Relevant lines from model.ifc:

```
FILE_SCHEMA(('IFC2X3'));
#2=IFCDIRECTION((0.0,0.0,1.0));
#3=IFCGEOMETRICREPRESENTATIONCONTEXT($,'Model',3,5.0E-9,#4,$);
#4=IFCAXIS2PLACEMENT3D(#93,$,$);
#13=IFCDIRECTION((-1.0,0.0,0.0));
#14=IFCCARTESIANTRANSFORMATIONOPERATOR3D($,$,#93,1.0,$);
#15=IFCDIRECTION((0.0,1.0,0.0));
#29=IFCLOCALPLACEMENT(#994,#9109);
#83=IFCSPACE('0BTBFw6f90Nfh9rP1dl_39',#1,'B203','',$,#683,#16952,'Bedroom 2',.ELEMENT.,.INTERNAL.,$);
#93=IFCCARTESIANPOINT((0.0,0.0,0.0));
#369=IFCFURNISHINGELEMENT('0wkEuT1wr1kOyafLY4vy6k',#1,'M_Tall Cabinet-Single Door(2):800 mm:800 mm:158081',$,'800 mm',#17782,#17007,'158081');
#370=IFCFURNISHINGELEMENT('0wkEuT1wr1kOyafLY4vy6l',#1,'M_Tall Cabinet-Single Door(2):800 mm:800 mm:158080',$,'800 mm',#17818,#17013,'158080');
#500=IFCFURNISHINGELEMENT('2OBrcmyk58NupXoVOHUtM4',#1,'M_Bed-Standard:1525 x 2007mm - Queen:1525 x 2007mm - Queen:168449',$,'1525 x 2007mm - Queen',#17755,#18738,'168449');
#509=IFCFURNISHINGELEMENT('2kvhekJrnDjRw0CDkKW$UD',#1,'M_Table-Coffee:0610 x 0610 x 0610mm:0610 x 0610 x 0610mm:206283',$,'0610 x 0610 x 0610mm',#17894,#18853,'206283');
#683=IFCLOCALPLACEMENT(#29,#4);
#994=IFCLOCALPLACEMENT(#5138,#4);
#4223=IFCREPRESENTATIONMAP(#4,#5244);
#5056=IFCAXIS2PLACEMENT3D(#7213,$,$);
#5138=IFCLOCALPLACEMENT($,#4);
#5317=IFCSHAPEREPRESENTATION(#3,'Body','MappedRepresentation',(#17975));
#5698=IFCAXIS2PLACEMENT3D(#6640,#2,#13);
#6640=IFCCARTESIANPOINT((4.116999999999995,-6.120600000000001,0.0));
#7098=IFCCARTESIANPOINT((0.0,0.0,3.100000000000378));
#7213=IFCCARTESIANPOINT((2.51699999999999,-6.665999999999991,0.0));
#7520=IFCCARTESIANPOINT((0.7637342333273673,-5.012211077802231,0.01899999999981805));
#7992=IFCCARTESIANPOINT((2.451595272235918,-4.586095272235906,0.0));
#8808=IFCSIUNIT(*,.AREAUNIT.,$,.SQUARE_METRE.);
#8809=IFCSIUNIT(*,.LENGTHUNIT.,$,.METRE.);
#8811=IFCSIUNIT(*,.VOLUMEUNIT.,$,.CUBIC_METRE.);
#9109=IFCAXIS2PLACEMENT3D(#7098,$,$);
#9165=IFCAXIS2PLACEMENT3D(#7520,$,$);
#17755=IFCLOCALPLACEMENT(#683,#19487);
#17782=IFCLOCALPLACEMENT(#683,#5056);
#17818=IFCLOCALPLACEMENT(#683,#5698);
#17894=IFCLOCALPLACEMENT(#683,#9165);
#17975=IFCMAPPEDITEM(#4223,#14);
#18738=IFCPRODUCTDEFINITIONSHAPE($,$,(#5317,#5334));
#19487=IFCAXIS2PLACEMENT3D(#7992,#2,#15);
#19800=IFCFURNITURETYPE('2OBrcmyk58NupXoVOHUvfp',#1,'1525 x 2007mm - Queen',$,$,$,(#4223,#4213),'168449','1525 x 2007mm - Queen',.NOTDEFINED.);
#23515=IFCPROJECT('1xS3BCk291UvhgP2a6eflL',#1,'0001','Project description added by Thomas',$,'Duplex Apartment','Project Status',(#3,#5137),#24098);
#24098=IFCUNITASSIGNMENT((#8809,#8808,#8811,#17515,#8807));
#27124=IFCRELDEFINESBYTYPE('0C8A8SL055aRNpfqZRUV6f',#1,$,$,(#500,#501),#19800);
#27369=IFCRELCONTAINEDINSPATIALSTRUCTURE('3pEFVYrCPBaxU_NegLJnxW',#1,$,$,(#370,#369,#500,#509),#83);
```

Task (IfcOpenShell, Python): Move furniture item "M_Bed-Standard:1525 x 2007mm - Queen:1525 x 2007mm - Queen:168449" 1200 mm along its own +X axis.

```python
import ifcopenshell
import ifcopenshell.api.geometry
import ifcopenshell.util.placement
import ifcopenshell.util.unit

model = ifcopenshell.open("model.ifc")
unit_scale = ifcopenshell.util.unit.calculate_unit_scale(model)

item = model.by_guid("2OBrcmyk58NupXoVOHUtM4")
matrix = ifcopenshell.util.placement.get_local_placement(item.ObjectPlacement)
matrix[:3, 3] += matrix[:3, 0] * 1.2 / unit_scale
ifcopenshell.api.geometry.edit_object_placement(model, product=item, matrix=matrix, is_si=False)

print(ifcopenshell.util.placement.get_local_placement(item.ObjectPlacement).round(3) + 0.0)

model.write("model-out.ifc")
```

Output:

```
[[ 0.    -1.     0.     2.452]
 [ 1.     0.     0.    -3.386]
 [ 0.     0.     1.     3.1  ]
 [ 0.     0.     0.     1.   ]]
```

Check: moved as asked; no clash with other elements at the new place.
